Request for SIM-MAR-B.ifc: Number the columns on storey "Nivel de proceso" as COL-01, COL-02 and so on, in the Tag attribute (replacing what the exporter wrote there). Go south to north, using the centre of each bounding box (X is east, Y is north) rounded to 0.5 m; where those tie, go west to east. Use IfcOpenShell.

First a look at what the model holds.

```python
import ifcopenshell
import ifcopenshell.util.element
import ifcopenshell.util.placement

model = ifcopenshell.open("SIM-MAR-B.ifc")
print(model.schema)
storey = next(s for s in model.by_type("IfcBuildingStorey") if s.Name == "Nivel de proceso")
columns = [e for e in ifcopenshell.util.element.get_decomposition(storey) if e.is_a("IfcColumn")]
for e in sorted(columns, key=lambda e: e.id()):
    origin = ifcopenshell.util.placement.get_local_placement(e.ObjectPlacement)[:3, 3]
    print(e.id(), e.Tag, e.Name, origin.round(2) + 0.0, sep=" | ")
```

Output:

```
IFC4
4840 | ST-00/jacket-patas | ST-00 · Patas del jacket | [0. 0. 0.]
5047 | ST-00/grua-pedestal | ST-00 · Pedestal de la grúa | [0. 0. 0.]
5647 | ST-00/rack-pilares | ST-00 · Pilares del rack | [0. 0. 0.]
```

```python
import ifcopenshell
import ifcopenshell.geom
import ifcopenshell.util.element
import ifcopenshell.util.shape

model = ifcopenshell.open("SIM-MAR-B.ifc")
settings = ifcopenshell.geom.settings()
settings.set("use-world-coords", True)


def centre(element):
    shape = ifcopenshell.geom.create_shape(settings, element)
    return ifcopenshell.util.shape.get_bbox_centroid(shape.geometry)


storey = next(s for s in model.by_type("IfcBuildingStorey") if s.Name == "Nivel de proceso")
columns = [e for e in ifcopenshell.util.element.get_decomposition(storey) if e.is_a("IfcColumn")]

# Insertion points can sit at a corner or the storey origin, so sort by the geometry (in metres).
centres = {e: centre(e) for e in columns}
columns.sort(key=lambda e: (round(centres[e][1] / 0.5), centres[e][0]))

for i, e in enumerate(columns, start=1):
    number = f"COL-{i:02d}"
    e.Tag = number
    print(e.id(), number)

model.write("SIM-MAR-B-out.ifc")
```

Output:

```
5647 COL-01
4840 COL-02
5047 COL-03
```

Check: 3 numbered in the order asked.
